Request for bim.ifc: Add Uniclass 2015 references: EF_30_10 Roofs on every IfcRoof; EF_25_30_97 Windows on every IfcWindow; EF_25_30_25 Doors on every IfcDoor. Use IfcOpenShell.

First a look at what the model holds.

```python
import ifcopenshell

model = ifcopenshell.open("bim.ifc")
print(model.schema)
print("classifications:", [c.Name for c in model.by_type("IfcClassification")])
for ifc_class in ("IfcDoor", "IfcRoof", "IfcStair", "IfcWall", "IfcWindow"):
    print(ifc_class, len(model.by_type(ifc_class)))
```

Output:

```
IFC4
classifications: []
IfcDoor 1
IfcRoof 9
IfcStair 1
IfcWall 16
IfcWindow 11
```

```python
import ifcopenshell
import ifcopenshell.api.classification

model = ifcopenshell.open("bim.ifc")

system = ifcopenshell.api.classification.add_classification(model, classification="Uniclass 2015")

codes = {
    "IfcRoof": ("EF_30_10", "Roofs"),
    "IfcWindow": ("EF_25_30_97", "Windows"),
    "IfcDoor": ("EF_25_30_25", "Doors"),
}
for ifc_class, (code, name) in codes.items():
    products = model.by_type(ifc_class)
    ifcopenshell.api.classification.add_reference(
        model, products=products, classification=system, identification=code, name=name
    )
    print(code, len(products))

model.write("bim_rev.ifc")
```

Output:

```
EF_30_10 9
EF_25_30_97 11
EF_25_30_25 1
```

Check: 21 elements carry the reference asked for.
